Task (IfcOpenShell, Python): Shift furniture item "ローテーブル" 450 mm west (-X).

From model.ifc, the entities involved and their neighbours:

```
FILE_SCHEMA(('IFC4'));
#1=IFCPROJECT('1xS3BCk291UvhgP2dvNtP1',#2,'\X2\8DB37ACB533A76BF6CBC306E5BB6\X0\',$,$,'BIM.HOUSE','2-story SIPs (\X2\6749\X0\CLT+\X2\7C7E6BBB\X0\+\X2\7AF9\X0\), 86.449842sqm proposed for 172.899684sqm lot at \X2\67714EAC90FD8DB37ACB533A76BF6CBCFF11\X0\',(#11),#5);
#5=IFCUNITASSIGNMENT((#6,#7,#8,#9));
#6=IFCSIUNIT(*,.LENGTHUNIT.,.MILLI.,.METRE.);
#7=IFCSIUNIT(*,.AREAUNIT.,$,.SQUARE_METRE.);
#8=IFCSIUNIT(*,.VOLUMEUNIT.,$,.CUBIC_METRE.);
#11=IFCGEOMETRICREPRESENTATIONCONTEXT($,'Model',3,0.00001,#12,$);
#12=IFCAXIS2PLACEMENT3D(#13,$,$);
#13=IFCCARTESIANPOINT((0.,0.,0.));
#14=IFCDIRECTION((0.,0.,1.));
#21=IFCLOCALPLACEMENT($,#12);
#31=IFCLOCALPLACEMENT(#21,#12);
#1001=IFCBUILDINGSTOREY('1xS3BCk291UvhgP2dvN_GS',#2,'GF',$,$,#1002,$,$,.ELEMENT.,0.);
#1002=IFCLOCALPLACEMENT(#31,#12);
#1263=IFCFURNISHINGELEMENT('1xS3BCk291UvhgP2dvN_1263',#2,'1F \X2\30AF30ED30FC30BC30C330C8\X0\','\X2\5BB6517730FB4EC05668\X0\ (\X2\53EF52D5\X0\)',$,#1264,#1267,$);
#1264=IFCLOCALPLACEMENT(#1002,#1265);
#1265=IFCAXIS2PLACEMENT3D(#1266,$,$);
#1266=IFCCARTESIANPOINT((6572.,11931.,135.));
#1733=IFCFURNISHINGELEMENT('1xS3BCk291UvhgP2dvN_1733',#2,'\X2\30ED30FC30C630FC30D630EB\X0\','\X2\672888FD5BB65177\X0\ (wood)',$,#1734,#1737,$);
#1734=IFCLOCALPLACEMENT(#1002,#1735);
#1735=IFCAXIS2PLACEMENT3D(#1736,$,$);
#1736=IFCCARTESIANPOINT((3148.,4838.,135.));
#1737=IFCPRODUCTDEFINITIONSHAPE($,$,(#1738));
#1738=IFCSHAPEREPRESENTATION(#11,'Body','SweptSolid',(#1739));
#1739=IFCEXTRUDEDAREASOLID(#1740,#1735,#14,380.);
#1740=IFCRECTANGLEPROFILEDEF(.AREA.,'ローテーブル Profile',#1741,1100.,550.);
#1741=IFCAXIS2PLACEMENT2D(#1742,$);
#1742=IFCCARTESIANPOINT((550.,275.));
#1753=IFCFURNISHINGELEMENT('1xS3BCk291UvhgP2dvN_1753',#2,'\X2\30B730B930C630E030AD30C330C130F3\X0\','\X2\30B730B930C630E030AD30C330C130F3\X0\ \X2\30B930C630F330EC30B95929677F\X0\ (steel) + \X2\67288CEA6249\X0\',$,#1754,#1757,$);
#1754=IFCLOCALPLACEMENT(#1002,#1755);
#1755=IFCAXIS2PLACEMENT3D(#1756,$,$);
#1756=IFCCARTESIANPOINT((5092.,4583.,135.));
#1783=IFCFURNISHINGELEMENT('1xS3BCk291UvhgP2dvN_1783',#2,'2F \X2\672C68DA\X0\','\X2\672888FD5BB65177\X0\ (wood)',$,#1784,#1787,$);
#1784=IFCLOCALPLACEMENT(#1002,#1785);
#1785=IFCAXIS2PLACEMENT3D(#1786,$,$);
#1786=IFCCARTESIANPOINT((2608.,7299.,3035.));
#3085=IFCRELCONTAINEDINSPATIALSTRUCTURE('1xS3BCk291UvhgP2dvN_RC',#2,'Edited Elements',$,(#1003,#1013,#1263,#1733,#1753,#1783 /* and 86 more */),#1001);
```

```python
import ifcopenshell
import ifcopenshell.api.geometry
import ifcopenshell.util.placement
import ifcopenshell.util.unit

model = ifcopenshell.open("model.ifc")
unit_scale = ifcopenshell.util.unit.calculate_unit_scale(model)

item = model.by_id(1733)
matrix = ifcopenshell.util.placement.get_local_placement(item.ObjectPlacement)
matrix[0, 3] -= 0.45 / unit_scale
ifcopenshell.api.geometry.edit_object_placement(model, product=item, matrix=matrix, is_si=False)

print(ifcopenshell.util.placement.get_local_placement(item.ObjectPlacement).round(3) + 0.0)

model.write("model_updated.ifc")
```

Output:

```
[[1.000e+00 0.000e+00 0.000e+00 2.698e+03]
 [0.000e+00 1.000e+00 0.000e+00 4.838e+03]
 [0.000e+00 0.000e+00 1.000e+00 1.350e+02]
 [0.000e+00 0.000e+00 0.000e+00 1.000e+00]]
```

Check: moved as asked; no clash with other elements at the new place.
